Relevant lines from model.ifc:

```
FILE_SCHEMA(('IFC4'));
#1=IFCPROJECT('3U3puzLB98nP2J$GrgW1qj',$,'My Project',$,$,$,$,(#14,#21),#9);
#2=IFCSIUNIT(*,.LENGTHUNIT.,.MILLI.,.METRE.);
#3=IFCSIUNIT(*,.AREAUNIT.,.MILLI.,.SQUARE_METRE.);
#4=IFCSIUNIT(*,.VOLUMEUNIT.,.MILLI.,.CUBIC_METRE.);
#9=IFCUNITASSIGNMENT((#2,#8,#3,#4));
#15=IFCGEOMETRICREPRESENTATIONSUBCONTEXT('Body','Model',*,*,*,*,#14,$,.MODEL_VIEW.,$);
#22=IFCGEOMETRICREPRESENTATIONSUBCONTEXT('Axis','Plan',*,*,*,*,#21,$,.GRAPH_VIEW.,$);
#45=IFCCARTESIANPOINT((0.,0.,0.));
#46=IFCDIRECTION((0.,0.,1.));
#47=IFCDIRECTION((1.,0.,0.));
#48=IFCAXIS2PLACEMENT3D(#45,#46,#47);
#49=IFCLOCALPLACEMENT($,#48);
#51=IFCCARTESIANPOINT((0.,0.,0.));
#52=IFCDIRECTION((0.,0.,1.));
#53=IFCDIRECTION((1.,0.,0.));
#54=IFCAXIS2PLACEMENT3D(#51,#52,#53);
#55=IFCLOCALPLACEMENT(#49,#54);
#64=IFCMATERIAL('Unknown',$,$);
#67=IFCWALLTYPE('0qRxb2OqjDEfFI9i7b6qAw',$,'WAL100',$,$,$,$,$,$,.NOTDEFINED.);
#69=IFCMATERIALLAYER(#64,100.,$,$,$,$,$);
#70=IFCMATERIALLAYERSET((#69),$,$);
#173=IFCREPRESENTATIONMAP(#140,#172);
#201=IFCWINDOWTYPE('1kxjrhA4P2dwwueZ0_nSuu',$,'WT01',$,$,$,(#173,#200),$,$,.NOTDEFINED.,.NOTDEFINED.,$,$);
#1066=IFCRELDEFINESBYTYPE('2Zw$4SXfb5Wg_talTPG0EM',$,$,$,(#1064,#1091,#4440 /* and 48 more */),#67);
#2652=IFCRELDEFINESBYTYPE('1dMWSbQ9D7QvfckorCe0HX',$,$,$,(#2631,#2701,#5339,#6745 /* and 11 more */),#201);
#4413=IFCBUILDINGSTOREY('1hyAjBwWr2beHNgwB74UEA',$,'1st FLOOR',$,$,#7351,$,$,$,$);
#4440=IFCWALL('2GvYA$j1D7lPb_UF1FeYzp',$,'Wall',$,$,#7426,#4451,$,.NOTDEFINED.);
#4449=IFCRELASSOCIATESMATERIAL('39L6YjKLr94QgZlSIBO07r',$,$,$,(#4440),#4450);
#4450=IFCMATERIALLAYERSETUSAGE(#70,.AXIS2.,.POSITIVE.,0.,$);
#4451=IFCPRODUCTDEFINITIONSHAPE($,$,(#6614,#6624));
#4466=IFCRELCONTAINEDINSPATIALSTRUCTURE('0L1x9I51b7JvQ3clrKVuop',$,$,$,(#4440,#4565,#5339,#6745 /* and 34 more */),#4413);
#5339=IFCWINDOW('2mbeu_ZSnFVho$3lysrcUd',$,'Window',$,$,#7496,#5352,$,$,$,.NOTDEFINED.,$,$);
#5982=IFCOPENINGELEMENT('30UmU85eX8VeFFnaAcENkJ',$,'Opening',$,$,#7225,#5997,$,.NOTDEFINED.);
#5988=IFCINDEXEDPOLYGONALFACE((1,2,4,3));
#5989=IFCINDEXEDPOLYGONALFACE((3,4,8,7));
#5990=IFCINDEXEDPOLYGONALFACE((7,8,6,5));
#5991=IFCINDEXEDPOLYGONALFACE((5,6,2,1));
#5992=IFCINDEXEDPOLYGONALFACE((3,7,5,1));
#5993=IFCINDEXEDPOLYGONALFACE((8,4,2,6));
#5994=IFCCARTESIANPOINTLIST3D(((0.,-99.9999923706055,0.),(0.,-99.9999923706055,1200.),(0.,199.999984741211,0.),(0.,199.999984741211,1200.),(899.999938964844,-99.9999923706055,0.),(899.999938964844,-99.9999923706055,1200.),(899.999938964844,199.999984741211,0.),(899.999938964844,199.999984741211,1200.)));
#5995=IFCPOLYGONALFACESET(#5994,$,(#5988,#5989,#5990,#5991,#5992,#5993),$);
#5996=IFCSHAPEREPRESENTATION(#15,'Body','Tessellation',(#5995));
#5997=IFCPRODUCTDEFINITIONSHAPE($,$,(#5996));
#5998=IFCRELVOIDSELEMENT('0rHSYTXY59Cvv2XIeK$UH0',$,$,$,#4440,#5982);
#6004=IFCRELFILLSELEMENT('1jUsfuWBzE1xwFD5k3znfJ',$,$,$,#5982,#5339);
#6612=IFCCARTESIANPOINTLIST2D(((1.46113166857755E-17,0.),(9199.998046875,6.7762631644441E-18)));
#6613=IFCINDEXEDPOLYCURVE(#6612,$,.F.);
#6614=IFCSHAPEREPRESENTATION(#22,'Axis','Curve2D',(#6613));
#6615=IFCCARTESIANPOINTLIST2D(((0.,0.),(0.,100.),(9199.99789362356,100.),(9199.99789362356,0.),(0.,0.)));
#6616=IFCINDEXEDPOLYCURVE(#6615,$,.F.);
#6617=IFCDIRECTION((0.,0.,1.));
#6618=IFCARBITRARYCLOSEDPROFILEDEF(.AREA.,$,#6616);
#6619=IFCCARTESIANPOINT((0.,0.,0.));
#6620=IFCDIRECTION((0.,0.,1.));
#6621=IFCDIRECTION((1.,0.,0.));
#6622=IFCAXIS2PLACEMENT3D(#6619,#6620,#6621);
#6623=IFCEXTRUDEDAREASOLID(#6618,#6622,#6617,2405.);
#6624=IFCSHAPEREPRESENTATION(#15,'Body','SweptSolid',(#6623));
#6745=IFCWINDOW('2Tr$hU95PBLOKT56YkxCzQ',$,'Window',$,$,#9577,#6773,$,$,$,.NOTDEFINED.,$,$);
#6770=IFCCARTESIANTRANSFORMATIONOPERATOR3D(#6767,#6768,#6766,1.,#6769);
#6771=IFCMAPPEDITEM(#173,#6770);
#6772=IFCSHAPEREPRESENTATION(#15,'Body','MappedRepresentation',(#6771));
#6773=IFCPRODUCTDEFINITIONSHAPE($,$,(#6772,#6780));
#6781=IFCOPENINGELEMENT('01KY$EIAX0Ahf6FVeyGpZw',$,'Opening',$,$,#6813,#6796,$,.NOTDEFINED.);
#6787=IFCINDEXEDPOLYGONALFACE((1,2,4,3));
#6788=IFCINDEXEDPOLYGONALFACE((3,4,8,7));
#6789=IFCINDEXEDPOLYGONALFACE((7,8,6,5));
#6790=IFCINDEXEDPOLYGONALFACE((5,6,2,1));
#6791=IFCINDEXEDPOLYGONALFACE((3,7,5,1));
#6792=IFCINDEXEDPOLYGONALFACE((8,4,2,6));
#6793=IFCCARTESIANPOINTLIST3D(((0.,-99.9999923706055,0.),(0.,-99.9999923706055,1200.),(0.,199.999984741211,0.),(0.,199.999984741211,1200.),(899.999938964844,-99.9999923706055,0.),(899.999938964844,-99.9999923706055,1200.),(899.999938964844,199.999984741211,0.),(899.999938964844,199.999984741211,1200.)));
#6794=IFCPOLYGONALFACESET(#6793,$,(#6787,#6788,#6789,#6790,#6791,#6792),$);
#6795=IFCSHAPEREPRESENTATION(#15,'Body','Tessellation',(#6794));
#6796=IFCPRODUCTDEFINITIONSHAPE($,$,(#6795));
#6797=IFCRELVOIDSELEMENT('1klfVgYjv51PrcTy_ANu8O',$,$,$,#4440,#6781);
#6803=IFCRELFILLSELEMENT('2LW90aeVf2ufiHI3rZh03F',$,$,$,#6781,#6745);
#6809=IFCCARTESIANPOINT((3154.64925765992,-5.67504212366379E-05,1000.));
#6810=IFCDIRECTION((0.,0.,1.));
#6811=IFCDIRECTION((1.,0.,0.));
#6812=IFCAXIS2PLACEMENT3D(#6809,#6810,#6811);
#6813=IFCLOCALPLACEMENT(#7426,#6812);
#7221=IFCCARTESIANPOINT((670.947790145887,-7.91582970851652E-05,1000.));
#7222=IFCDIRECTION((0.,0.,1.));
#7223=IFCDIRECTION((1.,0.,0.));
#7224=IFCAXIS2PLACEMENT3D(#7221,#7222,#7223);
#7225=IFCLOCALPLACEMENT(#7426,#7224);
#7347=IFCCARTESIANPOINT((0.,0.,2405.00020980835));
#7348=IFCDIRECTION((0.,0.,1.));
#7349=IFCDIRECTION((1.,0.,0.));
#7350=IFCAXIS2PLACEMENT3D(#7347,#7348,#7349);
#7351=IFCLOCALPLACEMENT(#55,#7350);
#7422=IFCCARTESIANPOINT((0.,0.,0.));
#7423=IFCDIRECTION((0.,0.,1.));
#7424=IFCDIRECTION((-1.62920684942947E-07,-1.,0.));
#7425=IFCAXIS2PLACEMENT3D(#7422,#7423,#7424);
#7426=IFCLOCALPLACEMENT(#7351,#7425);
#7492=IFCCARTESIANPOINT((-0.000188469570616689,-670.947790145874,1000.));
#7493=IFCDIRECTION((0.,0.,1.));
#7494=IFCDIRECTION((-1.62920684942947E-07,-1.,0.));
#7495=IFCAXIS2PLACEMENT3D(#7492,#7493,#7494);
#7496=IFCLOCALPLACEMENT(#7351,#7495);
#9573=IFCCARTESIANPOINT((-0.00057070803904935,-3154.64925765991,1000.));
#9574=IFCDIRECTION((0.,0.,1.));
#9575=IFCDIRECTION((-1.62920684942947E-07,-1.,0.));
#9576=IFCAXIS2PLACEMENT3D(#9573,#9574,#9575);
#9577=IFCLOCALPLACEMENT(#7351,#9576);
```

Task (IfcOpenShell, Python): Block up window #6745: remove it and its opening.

```python
import ifcopenshell
import ifcopenshell.api.feature
import ifcopenshell.api.root
import ifcopenshell.geom
import ifcopenshell.util.shape

model = ifcopenshell.open("model.ifc")
settings = ifcopenshell.geom.settings()


def volume(element):
    """Net volume in cubic metres, openings subtracted."""
    shape = ifcopenshell.geom.create_shape(settings, element)
    return ifcopenshell.util.shape.get_volume(shape.geometry)


window = model.by_guid("2Tr$hU95PBLOKT56YkxCzQ")
opening = window.FillsVoids[0].RelatingOpeningElement
wall = opening.VoidsElements[0].RelatingBuildingElement
before = volume(wall)

ifcopenshell.api.root.remove_product(model, product=window)
ifcopenshell.api.feature.remove_feature(model, feature=opening)

after = volume(wall)

print(f"wall volume {before:.3f} -> {after:.3f} m3")

model.write("model_edited.ifc")
```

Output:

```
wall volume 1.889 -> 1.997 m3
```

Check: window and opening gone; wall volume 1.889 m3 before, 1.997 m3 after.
